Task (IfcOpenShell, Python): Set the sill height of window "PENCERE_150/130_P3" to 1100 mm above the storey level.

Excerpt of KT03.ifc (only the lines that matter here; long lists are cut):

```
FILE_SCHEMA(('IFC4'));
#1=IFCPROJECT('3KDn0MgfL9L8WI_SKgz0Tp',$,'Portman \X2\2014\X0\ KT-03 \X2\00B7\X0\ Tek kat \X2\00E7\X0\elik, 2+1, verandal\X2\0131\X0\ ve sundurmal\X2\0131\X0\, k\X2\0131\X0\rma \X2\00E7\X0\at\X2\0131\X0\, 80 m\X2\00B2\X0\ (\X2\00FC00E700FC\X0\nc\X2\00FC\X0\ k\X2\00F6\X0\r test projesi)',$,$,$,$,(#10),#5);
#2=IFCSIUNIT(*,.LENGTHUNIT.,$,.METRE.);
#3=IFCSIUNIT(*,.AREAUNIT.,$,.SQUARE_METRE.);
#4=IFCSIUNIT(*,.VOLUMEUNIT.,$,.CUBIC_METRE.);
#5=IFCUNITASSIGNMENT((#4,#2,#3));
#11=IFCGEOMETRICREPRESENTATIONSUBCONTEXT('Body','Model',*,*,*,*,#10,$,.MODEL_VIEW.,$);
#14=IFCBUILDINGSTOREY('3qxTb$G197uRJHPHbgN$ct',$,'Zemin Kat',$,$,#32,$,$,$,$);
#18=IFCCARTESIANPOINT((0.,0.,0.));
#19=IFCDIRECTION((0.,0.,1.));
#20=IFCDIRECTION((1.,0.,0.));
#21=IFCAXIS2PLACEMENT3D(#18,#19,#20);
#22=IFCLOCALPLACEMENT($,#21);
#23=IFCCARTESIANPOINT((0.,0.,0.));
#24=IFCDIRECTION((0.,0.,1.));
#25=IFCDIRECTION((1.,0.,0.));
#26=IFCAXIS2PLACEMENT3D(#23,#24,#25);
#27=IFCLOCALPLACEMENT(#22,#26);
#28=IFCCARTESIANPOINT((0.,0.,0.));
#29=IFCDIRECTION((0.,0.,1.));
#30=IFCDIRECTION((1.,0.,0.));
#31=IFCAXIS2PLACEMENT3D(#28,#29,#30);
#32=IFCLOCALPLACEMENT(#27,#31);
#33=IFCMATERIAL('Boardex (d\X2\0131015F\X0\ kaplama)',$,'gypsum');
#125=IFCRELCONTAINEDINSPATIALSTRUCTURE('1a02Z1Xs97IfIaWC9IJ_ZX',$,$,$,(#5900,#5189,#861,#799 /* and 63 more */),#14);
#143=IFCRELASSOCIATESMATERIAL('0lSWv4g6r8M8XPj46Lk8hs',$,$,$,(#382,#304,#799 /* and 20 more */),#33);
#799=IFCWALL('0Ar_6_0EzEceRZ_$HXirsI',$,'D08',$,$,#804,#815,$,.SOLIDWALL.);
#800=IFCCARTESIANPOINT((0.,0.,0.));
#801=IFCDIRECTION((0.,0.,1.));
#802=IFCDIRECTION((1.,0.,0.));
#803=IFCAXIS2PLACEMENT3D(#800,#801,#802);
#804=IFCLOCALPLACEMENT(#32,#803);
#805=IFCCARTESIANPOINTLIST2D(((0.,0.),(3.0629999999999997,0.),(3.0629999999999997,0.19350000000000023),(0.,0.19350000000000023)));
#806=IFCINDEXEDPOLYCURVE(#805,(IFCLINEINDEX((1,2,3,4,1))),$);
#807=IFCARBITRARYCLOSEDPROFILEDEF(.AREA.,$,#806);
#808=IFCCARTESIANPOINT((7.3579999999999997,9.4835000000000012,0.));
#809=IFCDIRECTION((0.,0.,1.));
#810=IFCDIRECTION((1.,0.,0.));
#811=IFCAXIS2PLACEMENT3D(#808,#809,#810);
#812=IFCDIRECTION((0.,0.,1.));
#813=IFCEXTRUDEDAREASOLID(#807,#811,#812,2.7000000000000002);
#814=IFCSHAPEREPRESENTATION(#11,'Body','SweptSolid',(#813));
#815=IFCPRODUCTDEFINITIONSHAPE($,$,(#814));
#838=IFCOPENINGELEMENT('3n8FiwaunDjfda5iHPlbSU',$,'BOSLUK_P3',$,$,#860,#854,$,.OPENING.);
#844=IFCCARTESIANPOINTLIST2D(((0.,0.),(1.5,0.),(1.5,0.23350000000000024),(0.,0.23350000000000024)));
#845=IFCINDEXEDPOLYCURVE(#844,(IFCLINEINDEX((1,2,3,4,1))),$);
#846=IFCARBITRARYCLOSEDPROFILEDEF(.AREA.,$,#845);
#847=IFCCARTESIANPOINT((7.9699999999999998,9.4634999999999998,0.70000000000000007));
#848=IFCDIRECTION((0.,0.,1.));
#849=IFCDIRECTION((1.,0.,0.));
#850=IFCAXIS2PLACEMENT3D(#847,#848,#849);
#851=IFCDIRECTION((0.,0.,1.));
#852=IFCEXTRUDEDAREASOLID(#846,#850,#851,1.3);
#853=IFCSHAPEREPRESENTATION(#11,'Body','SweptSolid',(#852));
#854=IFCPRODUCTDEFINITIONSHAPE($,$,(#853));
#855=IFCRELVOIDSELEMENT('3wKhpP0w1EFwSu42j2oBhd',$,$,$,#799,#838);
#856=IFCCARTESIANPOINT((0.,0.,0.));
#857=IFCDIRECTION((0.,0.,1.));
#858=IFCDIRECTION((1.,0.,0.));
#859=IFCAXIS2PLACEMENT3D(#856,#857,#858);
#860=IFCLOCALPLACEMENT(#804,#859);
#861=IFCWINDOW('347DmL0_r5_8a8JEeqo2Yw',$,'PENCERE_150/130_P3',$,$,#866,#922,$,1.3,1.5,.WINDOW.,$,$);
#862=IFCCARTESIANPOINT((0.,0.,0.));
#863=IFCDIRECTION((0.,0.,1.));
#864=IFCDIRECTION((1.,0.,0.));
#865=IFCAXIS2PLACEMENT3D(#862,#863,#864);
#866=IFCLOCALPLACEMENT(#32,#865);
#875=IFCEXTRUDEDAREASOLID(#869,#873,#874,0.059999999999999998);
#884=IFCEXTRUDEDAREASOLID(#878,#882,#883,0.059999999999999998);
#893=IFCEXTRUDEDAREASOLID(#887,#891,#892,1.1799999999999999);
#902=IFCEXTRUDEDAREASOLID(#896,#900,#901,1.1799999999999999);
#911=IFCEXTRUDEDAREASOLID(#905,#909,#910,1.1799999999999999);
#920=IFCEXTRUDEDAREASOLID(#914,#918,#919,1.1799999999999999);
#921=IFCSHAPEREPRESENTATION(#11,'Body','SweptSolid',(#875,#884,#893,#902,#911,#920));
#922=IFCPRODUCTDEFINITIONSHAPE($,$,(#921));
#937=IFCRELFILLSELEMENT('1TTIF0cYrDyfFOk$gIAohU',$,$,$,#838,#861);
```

```python
import numpy as np
import ifcopenshell
import ifcopenshell.api.geometry
import ifcopenshell.geom
import ifcopenshell.util.element
import ifcopenshell.util.placement
import ifcopenshell.util.shape
import ifcopenshell.util.unit

model = ifcopenshell.open("KT03.ifc")
unit_scale = ifcopenshell.util.unit.calculate_unit_scale(model)

window = model.by_guid("347DmL0_r5_8a8JEeqo2Yw")
opening = window.FillsVoids[0].RelatingOpeningElement
storey = ifcopenshell.util.element.get_container(window, ifc_class="IfcBuildingStorey")
level = ifcopenshell.util.placement.get_local_placement(storey.ObjectPlacement)[2, 3]

# The opening's origin need not be at the sill, so measure its lowest point.
shape = ifcopenshell.geom.create_shape(ifcopenshell.geom.settings(), opening)
bottom = ifcopenshell.util.shape.get_shape_bottom_elevation(shape, shape.geometry) / unit_scale
dz = level + 1.1 / unit_scale - bottom

shift = np.array([0.0, 0.0, dz])
# The window is not placed relative to its opening, so move both.
for product in (opening, window):
    matrix = ifcopenshell.util.placement.get_local_placement(product.ObjectPlacement)
    matrix[:3, 3] += shift
    ifcopenshell.api.geometry.edit_object_placement(model, product=product, matrix=matrix, is_si=False)

print(f"moved by {dz * unit_scale:+.3f} m")

model.write("KT03_edited.ifc")
```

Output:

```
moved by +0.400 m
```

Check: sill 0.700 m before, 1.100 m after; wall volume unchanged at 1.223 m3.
